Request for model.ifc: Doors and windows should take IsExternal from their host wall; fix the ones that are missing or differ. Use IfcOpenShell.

First a look at what the model holds.

```python
import ifcopenshell
import ifcopenshell.util.element

model = ifcopenshell.open("model.ifc")
print(model.schema)
seen = {}
for e in model.by_type("IfcDoor") + model.by_type("IfcWindow"):
    if not e.FillsVoids:
        continue
    host = e.FillsVoids[0].RelatingOpeningElement.VoidsElements[0].RelatingBuildingElement
    own = ifcopenshell.util.element.get_pset(e, f"Pset_{e.is_a()[3:].removesuffix('StandardCase')}Common", "IsExternal")
    wall = ifcopenshell.util.element.get_pset(host, "Pset_WallCommon", "IsExternal")
    seen[e.is_a(), own, wall] = seen.get((e.is_a(), own, wall), 0) + 1
for (cls, own, wall), count in sorted(seen.items(), key=str):
    print(count, cls, "IsExternal:", own, "| host wall:", wall)
```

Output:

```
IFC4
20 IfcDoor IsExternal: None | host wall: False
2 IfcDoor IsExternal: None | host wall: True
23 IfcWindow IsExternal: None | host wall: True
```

```python
import ifcopenshell
import ifcopenshell.api.pset
import ifcopenshell.util.element

model = ifcopenshell.open("model.ifc")

count = 0
for ifc_class, pset_name in (("IfcDoor", "Pset_DoorCommon"), ("IfcWindow", "Pset_WindowCommon")):
    for e in model.by_type(ifc_class):
        if not e.FillsVoids:
            continue
        host = e.FillsVoids[0].RelatingOpeningElement.VoidsElements[0].RelatingBuildingElement
        external = ifcopenshell.util.element.get_pset(host, "Pset_WallCommon", "IsExternal")
        if external is None or ifcopenshell.util.element.get_pset(e, pset_name, "IsExternal") == external:
            continue
        pset = ifcopenshell.api.pset.add_pset(model, product=e, name=pset_name)
        ifcopenshell.api.pset.edit_pset(model, pset=pset, properties={"IsExternal": external})
        count += 1

print(count, "updated")

model.write("model_v2.ifc")
```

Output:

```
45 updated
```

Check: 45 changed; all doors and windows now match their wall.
